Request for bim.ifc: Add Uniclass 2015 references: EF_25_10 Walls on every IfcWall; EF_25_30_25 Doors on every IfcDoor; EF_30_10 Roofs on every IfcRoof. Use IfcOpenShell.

First a look at what the model holds.

```python
import ifcopenshell

model = ifcopenshell.open("bim.ifc")
print(model.schema)
print("classifications:", [c.Name for c in model.by_type("IfcClassification")])
for ifc_class in ("IfcDoor", "IfcRoof", "IfcStair", "IfcWall", "IfcWindow"):
    print(ifc_class, len(model.by_type(ifc_class)))
```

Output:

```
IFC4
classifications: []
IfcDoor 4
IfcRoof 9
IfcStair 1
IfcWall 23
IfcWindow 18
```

```python
import ifcopenshell
import ifcopenshell.api.classification

model = ifcopenshell.open("bim.ifc")

system = ifcopenshell.api.classification.add_classification(model, classification="Uniclass 2015")

codes = {
    "IfcWall": ("EF_25_10", "Walls"),
    "IfcDoor": ("EF_25_30_25", "Doors"),
    "IfcRoof": ("EF_30_10", "Roofs"),
}
for ifc_class, (code, name) in codes.items():
    products = model.by_type(ifc_class)
    ifcopenshell.api.classification.add_reference(
        model, products=products, classification=system, identification=code, name=name
    )
    print(code, len(products))

model.write("bim_rev.ifc")
```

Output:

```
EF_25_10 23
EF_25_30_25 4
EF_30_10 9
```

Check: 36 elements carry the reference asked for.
